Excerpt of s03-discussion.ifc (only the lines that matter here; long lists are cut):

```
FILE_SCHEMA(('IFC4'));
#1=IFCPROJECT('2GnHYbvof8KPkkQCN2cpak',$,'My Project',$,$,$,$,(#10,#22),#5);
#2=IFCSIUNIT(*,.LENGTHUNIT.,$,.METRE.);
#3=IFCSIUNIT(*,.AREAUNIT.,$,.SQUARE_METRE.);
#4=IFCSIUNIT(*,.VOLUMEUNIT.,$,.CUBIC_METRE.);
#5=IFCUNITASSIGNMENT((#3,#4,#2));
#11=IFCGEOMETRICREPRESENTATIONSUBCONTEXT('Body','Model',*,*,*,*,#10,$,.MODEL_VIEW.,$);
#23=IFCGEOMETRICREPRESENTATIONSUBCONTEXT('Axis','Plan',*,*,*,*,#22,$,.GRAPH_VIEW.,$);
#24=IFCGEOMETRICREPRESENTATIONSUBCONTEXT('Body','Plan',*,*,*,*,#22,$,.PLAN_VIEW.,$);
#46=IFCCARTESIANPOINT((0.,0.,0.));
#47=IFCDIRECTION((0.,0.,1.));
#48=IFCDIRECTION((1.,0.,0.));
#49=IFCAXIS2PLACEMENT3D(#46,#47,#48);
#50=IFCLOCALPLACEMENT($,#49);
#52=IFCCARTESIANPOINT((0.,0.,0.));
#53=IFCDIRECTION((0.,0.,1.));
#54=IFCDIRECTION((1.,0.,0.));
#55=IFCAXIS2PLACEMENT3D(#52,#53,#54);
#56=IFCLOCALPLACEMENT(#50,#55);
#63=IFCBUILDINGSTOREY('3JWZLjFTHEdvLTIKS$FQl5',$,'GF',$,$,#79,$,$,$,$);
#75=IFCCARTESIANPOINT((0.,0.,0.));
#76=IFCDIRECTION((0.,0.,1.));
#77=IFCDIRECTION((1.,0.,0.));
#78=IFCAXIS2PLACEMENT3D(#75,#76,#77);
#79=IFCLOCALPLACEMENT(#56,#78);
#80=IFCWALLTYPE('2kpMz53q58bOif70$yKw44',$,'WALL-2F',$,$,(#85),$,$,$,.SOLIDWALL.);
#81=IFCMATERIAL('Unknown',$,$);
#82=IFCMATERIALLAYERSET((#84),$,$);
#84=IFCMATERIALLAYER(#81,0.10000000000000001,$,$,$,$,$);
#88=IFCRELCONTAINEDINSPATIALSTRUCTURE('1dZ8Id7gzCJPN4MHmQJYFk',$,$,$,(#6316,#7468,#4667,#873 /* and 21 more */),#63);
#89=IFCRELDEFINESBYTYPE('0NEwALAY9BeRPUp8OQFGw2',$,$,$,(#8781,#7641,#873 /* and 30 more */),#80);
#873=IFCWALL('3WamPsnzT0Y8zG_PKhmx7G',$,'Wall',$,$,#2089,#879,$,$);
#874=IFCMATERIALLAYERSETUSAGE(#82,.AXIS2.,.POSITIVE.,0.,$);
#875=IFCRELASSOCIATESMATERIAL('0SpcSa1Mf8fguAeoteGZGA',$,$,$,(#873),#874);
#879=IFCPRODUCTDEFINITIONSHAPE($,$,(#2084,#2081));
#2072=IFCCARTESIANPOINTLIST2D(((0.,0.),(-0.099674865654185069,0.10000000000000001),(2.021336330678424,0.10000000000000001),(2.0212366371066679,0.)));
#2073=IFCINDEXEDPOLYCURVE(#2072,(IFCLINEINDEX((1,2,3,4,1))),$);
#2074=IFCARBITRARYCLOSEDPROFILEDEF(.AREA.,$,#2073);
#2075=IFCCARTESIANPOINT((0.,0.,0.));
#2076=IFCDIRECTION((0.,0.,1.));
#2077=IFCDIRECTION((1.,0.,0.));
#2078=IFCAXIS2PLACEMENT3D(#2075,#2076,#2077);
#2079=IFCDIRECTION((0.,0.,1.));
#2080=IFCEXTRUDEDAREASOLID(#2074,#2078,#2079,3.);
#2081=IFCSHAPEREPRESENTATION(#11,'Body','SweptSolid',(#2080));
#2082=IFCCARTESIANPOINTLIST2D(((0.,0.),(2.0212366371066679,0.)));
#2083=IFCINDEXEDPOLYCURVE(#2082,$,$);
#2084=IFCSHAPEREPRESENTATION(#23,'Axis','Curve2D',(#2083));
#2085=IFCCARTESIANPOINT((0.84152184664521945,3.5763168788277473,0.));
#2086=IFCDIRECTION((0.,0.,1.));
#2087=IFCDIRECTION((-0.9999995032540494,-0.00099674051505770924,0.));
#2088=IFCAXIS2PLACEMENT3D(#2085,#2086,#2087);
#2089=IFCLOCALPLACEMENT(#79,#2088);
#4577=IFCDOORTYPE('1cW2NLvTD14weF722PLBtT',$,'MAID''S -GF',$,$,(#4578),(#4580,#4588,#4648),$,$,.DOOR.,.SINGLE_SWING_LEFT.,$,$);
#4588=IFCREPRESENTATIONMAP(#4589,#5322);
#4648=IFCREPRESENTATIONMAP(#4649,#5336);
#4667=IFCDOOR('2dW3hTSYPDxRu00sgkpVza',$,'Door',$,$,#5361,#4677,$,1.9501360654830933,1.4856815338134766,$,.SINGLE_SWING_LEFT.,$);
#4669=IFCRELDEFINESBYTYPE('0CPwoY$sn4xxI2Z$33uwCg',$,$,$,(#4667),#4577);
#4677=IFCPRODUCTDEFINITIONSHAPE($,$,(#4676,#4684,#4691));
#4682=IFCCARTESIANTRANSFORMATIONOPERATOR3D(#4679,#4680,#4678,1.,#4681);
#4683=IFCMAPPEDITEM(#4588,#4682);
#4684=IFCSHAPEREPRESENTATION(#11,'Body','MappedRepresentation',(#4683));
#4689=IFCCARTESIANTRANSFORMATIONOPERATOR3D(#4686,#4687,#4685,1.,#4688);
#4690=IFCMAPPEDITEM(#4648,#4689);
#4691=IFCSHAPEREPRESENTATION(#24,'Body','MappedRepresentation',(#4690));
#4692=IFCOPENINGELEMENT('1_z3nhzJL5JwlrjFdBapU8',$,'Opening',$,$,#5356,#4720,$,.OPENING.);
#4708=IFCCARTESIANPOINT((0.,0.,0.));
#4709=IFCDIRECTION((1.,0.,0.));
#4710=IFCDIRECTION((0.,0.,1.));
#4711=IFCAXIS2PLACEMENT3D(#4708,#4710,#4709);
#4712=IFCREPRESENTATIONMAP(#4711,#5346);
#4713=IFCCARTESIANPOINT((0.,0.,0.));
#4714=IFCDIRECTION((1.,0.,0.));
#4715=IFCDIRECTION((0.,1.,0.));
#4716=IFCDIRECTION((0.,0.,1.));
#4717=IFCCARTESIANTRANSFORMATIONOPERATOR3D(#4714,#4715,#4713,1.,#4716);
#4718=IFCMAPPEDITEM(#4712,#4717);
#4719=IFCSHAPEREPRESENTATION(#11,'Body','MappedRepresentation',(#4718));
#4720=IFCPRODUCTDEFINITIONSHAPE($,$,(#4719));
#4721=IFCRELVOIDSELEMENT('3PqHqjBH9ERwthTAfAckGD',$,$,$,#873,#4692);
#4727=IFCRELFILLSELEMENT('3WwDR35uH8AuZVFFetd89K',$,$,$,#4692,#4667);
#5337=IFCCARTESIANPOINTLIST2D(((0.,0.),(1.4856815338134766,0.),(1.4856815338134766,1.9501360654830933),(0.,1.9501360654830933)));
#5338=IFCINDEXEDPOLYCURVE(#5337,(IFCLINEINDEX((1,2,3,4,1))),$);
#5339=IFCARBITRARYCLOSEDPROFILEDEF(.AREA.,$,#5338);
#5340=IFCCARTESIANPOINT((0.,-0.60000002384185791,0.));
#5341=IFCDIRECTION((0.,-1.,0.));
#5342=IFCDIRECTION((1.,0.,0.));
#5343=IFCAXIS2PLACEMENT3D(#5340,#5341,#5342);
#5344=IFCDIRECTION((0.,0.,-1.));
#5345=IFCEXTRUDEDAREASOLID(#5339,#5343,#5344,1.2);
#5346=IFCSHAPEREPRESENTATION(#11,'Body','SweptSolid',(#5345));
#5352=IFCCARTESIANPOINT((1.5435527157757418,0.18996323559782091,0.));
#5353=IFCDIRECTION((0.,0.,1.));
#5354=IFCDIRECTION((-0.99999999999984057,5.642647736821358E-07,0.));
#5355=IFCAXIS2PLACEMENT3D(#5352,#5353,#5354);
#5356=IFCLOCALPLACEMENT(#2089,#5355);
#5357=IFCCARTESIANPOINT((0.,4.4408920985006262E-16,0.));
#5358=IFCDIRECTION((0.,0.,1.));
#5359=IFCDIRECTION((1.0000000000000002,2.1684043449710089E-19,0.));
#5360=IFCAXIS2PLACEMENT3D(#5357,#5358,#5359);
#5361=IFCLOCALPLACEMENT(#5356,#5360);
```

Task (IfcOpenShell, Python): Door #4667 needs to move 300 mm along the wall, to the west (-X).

```python
import ifcopenshell
import ifcopenshell.api.geometry
import ifcopenshell.util.placement
import ifcopenshell.util.unit

model = ifcopenshell.open("s03-discussion.ifc")
unit_scale = ifcopenshell.util.unit.calculate_unit_scale(model)

door = model.by_id(4667)
opening = door.FillsVoids[0].RelatingOpeningElement
wall = opening.VoidsElements[0].RelatingBuildingElement

wall_matrix = ifcopenshell.util.placement.get_local_placement(wall.ObjectPlacement)
shift = wall_matrix[:3, 0] * 0.3 / unit_scale
before = ifcopenshell.util.placement.get_local_placement(door.ObjectPlacement)[:3, 3].copy()

# The door is placed relative to its opening, so it follows when the opening moves.
matrix = ifcopenshell.util.placement.get_local_placement(opening.ObjectPlacement)
matrix[:3, 3] += shift
ifcopenshell.api.geometry.edit_object_placement(
    model, product=opening, matrix=matrix, is_si=False, should_transform_children=True
)

after = ifcopenshell.util.placement.get_local_placement(door.ObjectPlacement)[:3, 3]
print("door moved by", (after - before).round(3) + 0.0)

model.write("s03-discussion_edited.ifc")
```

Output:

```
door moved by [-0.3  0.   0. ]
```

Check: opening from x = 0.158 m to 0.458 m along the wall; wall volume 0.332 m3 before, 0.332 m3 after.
